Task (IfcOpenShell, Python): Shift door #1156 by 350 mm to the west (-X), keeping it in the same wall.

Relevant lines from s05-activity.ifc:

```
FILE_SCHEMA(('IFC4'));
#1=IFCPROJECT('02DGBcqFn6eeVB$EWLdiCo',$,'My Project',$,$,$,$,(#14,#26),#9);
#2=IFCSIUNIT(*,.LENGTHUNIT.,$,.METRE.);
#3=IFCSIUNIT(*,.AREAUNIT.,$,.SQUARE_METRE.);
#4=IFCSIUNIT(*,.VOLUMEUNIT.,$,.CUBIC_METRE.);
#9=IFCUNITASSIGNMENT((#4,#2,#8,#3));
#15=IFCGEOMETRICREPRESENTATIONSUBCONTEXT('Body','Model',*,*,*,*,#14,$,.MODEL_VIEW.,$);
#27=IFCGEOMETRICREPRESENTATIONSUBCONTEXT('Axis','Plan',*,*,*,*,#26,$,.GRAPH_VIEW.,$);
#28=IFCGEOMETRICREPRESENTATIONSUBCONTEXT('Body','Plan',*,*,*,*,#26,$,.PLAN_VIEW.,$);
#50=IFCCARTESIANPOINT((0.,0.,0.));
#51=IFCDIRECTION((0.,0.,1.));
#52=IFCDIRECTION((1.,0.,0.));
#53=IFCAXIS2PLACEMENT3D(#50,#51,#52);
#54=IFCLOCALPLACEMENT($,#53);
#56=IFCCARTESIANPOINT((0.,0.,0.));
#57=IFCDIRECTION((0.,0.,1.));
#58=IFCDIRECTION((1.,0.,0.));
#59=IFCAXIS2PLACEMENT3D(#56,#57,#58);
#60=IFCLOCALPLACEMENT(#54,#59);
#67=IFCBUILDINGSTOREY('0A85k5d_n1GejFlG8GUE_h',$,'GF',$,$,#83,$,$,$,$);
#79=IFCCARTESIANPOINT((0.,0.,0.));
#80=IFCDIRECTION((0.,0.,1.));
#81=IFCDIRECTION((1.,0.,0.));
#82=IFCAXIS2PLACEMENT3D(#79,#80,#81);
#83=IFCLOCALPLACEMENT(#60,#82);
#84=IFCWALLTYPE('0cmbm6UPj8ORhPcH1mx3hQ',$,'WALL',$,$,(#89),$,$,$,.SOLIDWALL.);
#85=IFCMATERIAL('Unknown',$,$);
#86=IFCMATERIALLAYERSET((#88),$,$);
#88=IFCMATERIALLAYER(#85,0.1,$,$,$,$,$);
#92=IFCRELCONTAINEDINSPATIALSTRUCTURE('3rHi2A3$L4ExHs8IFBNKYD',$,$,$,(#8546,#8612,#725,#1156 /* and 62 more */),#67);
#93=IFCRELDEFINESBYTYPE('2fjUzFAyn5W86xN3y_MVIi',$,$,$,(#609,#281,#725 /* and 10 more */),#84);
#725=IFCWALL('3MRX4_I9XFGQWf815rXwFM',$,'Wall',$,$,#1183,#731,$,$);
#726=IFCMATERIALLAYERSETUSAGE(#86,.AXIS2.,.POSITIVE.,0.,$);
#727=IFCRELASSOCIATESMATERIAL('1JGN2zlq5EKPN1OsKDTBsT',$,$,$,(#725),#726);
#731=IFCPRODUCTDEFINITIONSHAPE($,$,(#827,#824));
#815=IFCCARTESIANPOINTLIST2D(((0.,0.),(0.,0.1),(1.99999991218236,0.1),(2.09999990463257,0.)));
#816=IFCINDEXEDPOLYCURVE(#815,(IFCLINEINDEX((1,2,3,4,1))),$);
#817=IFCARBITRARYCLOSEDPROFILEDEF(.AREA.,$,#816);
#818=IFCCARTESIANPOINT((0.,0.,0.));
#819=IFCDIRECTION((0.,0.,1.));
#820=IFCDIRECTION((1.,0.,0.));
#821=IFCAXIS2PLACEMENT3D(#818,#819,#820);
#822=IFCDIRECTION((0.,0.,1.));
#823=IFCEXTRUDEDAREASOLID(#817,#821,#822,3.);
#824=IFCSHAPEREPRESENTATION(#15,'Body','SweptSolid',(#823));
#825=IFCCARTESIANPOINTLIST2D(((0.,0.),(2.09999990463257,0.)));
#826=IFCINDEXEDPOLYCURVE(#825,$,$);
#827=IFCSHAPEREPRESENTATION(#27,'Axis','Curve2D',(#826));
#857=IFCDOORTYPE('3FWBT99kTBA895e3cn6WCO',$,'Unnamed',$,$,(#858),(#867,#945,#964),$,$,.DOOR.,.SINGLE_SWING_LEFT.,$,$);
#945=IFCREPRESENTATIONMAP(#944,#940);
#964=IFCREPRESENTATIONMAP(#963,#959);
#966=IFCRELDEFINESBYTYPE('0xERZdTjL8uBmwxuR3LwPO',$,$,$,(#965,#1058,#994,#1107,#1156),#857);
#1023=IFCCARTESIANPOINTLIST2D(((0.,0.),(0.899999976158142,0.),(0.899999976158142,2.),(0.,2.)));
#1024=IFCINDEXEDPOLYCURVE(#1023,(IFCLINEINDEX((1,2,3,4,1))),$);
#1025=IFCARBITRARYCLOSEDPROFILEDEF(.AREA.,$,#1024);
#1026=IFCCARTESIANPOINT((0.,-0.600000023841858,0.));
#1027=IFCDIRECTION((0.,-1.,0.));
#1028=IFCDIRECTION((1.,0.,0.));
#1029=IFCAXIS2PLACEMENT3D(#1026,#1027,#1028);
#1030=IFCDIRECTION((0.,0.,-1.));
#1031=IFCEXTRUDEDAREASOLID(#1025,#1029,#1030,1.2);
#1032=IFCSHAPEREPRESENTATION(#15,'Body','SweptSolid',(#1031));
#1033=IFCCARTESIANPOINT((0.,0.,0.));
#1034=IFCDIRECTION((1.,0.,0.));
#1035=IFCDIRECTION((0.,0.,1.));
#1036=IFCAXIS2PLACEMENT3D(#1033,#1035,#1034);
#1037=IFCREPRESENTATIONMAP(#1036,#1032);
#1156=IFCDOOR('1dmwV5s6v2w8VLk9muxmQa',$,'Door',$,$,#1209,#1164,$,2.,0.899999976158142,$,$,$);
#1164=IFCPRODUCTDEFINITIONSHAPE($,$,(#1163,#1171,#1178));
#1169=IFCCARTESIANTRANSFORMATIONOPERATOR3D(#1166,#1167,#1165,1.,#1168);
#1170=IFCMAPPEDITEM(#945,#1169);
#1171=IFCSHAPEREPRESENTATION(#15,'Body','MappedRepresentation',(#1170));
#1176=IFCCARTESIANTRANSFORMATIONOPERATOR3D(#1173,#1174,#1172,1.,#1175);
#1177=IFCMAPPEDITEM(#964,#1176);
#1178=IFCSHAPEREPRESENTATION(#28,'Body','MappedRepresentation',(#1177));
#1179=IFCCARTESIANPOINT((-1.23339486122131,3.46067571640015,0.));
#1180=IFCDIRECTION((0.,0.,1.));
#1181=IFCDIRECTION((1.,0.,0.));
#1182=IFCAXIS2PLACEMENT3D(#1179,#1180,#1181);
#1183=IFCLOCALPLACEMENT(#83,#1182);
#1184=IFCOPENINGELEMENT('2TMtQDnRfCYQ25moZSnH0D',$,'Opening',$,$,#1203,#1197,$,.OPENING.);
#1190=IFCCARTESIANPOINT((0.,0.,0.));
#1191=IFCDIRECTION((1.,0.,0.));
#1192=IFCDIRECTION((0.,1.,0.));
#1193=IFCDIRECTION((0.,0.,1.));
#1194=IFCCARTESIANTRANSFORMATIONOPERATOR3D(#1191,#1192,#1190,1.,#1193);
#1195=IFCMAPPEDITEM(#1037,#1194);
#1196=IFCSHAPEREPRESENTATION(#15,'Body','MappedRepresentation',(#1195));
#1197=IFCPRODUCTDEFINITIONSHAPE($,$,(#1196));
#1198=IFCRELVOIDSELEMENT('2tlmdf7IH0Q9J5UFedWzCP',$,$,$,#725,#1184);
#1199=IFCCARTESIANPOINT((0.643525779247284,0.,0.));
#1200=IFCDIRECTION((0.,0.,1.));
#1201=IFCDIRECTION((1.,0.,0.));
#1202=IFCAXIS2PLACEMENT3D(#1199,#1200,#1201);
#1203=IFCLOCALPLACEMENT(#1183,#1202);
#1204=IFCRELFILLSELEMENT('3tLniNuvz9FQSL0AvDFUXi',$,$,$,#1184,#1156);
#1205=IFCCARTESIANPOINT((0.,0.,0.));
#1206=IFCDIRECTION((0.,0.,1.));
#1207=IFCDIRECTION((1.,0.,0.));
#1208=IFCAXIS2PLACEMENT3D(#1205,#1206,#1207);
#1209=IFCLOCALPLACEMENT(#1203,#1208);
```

```python
import ifcopenshell
import ifcopenshell.api.geometry
import ifcopenshell.util.placement
import ifcopenshell.util.unit

model = ifcopenshell.open("s05-activity.ifc")
unit_scale = ifcopenshell.util.unit.calculate_unit_scale(model)

door = model.by_guid("1dmwV5s6v2w8VLk9muxmQa")
opening = door.FillsVoids[0].RelatingOpeningElement
wall = opening.VoidsElements[0].RelatingBuildingElement

wall_matrix = ifcopenshell.util.placement.get_local_placement(wall.ObjectPlacement)
shift = wall_matrix[:3, 0] * -0.35 / unit_scale
before = ifcopenshell.util.placement.get_local_placement(door.ObjectPlacement)[:3, 3].copy()

# The door is placed relative to its opening, so it follows when the opening moves.
matrix = ifcopenshell.util.placement.get_local_placement(opening.ObjectPlacement)
matrix[:3, 3] += shift
ifcopenshell.api.geometry.edit_object_placement(
    model, product=opening, matrix=matrix, is_si=False, should_transform_children=True
)

after = ifcopenshell.util.placement.get_local_placement(door.ObjectPlacement)[:3, 3]
print("door moved by", (after - before).round(3) + 0.0)

model.write("s05-activity-out.ifc")
```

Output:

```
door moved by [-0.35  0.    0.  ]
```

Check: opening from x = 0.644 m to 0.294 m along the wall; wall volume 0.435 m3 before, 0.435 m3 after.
